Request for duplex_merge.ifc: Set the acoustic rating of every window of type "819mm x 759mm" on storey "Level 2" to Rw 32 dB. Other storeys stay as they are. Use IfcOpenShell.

First a look at what the model holds.

```python
import ifcopenshell
import ifcopenshell.util.element

model = ifcopenshell.open("duplex_merge.ifc")
print(model.schema)
storey = next(s for s in model.by_type("IfcBuildingStorey") if s.Name == "Level 2")
windows = [e for e in ifcopenshell.util.element.get_decomposition(storey) if e.is_a("IfcWindow")]
seen = {}
for e in windows:
    element_type = ifcopenshell.util.element.get_type(e)
    key = (element_type.Name if element_type != e and element_type else None, ifcopenshell.util.element.get_pset(e, "Pset_WindowCommon", "AcousticRating"))
    seen[key] = seen.get(key, 0) + 1
for (name, value), count in sorted(seen.items(), key=str):
    print(count, "x", name, "|", value)
```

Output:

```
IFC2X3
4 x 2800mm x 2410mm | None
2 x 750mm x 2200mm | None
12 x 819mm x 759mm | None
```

```python
import ifcopenshell
import ifcopenshell.api.pset
import ifcopenshell.util.element

model = ifcopenshell.open("duplex_merge.ifc")

storey = next(s for s in model.by_type("IfcBuildingStorey") if s.Name == "Level 2")
windows = [e for e in ifcopenshell.util.element.get_decomposition(storey) if e.is_a("IfcWindow")]

count = 0
for e in windows:
    element_type = ifcopenshell.util.element.get_type(e)
    if element_type in (None, e) or element_type.Name != "819mm x 759mm":
        continue
    # add_pset returns the element's existing set when there is one.
    pset = ifcopenshell.api.pset.add_pset(model, product=e, name="Pset_WindowCommon")
    ifcopenshell.api.pset.edit_pset(model, pset=pset, properties={"AcousticRating": "Rw 32 dB"})
    count += 1

print(count, "windows updated")

model.write("duplex_merge-out.ifc")
```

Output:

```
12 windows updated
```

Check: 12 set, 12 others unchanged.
